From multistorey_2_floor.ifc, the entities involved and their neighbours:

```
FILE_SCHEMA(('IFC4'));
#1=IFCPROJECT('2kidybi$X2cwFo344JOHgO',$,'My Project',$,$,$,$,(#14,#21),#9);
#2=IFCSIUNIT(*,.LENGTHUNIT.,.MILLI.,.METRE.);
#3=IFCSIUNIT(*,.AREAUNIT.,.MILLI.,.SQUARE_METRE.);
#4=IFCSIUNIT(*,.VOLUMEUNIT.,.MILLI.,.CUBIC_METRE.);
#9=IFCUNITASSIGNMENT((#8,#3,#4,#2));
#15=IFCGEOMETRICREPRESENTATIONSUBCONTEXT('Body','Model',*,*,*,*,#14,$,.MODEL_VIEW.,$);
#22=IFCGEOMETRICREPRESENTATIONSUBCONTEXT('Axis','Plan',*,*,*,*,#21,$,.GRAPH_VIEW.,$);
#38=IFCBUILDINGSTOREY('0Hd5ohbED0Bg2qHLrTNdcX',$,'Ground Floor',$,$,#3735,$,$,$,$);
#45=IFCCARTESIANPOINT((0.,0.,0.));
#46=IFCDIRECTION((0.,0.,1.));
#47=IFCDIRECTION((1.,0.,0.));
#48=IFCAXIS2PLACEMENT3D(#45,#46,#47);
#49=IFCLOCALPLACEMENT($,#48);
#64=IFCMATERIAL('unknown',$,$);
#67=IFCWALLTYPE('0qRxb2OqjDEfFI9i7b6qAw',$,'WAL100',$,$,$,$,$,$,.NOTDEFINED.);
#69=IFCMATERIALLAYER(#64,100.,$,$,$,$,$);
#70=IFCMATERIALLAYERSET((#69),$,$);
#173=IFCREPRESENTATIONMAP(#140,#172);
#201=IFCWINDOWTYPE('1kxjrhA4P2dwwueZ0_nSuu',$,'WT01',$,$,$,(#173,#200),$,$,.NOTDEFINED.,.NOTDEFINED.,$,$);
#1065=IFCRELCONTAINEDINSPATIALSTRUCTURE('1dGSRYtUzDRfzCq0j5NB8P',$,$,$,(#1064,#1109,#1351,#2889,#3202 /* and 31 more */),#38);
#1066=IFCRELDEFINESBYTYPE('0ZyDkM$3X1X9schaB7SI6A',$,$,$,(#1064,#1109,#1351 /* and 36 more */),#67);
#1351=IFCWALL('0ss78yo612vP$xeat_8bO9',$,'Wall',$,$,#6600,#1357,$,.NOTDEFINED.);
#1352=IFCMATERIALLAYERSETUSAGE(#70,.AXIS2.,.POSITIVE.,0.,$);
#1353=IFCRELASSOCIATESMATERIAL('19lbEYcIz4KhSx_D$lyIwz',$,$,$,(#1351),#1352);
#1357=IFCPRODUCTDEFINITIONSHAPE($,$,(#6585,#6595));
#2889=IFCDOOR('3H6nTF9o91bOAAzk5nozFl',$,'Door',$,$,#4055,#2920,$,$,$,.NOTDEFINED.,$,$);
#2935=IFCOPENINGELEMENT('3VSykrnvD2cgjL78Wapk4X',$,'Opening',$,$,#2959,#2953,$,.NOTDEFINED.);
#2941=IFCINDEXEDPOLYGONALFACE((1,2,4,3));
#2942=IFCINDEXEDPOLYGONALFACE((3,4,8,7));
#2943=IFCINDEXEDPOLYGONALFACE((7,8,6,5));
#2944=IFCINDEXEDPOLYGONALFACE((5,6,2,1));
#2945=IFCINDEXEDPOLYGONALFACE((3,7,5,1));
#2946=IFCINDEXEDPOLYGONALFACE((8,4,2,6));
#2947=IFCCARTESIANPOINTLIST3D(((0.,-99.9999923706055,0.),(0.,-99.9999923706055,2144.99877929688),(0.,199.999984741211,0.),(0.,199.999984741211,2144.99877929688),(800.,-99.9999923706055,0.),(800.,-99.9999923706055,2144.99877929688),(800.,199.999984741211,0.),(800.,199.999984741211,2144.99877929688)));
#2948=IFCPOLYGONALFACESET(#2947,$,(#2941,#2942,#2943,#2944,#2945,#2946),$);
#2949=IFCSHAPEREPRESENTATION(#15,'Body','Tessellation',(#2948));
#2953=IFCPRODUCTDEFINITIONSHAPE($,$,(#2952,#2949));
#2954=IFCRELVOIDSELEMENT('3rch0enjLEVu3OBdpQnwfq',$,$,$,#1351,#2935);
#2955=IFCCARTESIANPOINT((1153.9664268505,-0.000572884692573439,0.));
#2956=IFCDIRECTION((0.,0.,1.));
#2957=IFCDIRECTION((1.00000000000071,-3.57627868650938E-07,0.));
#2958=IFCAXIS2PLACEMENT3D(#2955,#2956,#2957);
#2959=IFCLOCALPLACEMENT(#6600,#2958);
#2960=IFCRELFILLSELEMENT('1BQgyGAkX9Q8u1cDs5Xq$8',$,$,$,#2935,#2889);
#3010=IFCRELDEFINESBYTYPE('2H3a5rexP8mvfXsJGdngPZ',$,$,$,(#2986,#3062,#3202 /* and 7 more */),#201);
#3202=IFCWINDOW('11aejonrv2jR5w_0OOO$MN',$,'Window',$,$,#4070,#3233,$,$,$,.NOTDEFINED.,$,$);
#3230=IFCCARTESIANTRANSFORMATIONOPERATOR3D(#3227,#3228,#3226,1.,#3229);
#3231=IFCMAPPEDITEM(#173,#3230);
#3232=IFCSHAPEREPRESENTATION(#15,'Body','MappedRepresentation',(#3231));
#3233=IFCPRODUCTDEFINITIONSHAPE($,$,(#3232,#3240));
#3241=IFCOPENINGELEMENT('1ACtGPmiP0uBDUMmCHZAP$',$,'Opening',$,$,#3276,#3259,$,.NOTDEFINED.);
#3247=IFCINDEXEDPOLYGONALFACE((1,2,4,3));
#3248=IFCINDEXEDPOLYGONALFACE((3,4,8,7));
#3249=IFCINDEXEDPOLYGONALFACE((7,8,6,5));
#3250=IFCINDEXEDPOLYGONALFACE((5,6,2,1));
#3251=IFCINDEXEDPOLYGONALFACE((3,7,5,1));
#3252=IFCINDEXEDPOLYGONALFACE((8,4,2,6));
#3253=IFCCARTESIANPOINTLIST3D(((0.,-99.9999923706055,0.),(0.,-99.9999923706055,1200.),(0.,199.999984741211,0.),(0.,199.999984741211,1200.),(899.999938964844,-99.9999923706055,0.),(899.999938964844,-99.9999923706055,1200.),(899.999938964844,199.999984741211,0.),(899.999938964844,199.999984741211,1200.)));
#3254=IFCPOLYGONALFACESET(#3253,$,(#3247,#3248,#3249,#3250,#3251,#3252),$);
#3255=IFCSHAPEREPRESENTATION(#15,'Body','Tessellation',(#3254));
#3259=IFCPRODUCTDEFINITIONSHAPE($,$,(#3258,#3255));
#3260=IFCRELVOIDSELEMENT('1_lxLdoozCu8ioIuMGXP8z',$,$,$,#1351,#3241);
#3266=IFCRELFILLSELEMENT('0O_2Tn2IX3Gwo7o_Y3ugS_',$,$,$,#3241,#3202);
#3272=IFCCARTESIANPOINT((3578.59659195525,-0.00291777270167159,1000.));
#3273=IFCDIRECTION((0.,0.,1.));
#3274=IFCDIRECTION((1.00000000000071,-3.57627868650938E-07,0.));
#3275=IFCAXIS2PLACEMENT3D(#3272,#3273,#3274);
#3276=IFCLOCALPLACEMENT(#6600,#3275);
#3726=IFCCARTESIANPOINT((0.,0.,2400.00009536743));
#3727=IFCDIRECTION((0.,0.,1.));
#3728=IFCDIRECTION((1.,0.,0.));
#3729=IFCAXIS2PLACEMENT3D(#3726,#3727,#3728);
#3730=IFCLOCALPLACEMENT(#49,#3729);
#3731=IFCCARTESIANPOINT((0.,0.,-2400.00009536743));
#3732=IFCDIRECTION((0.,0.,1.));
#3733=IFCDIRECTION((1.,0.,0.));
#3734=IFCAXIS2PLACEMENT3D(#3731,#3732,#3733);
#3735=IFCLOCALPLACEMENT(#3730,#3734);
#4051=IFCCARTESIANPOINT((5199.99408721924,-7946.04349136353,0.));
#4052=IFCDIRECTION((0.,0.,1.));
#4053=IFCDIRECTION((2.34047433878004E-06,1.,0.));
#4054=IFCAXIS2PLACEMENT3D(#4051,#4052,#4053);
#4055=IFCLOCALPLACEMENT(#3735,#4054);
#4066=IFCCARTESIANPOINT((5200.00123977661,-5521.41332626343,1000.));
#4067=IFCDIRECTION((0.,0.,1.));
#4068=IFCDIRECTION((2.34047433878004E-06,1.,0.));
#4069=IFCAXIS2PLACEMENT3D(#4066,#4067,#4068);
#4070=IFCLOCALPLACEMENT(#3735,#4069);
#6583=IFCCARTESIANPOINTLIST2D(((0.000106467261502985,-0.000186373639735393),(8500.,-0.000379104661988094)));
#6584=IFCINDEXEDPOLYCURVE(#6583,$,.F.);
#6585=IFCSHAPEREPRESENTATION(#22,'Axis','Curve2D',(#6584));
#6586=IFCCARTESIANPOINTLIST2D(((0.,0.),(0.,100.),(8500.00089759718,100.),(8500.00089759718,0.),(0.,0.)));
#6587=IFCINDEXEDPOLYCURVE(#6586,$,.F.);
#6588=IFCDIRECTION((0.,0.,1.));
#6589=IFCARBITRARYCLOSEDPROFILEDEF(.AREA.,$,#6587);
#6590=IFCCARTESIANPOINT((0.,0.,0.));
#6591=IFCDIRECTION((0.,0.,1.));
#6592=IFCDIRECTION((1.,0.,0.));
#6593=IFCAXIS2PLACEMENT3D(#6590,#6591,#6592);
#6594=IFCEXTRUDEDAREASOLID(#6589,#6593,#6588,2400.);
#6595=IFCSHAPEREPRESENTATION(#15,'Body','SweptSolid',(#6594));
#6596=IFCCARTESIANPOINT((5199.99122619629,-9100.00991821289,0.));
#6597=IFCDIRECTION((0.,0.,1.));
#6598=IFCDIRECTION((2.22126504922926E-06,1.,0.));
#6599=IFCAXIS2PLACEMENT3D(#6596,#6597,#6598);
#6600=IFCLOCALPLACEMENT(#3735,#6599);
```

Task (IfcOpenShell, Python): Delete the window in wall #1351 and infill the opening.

```python
import ifcopenshell
import ifcopenshell.api.feature
import ifcopenshell.api.root
import ifcopenshell.geom
import ifcopenshell.util.shape

model = ifcopenshell.open("multistorey_2_floor.ifc")
settings = ifcopenshell.geom.settings()


def volume(element):
    """Net volume in cubic metres, openings subtracted."""
    shape = ifcopenshell.geom.create_shape(settings, element)
    return ifcopenshell.util.shape.get_volume(shape.geometry)


window = model.by_guid("11aejonrv2jR5w_0OOO$MN")
opening = window.FillsVoids[0].RelatingOpeningElement
wall = opening.VoidsElements[0].RelatingBuildingElement
before = volume(wall)

ifcopenshell.api.root.remove_product(model, product=window)
ifcopenshell.api.feature.remove_feature(model, feature=opening)

after = volume(wall)

print(f"wall volume {before:.3f} -> {after:.3f} m3")

model.write("multistorey_2_floor_rev.ifc")
```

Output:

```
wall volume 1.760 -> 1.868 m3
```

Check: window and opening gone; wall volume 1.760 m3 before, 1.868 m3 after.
